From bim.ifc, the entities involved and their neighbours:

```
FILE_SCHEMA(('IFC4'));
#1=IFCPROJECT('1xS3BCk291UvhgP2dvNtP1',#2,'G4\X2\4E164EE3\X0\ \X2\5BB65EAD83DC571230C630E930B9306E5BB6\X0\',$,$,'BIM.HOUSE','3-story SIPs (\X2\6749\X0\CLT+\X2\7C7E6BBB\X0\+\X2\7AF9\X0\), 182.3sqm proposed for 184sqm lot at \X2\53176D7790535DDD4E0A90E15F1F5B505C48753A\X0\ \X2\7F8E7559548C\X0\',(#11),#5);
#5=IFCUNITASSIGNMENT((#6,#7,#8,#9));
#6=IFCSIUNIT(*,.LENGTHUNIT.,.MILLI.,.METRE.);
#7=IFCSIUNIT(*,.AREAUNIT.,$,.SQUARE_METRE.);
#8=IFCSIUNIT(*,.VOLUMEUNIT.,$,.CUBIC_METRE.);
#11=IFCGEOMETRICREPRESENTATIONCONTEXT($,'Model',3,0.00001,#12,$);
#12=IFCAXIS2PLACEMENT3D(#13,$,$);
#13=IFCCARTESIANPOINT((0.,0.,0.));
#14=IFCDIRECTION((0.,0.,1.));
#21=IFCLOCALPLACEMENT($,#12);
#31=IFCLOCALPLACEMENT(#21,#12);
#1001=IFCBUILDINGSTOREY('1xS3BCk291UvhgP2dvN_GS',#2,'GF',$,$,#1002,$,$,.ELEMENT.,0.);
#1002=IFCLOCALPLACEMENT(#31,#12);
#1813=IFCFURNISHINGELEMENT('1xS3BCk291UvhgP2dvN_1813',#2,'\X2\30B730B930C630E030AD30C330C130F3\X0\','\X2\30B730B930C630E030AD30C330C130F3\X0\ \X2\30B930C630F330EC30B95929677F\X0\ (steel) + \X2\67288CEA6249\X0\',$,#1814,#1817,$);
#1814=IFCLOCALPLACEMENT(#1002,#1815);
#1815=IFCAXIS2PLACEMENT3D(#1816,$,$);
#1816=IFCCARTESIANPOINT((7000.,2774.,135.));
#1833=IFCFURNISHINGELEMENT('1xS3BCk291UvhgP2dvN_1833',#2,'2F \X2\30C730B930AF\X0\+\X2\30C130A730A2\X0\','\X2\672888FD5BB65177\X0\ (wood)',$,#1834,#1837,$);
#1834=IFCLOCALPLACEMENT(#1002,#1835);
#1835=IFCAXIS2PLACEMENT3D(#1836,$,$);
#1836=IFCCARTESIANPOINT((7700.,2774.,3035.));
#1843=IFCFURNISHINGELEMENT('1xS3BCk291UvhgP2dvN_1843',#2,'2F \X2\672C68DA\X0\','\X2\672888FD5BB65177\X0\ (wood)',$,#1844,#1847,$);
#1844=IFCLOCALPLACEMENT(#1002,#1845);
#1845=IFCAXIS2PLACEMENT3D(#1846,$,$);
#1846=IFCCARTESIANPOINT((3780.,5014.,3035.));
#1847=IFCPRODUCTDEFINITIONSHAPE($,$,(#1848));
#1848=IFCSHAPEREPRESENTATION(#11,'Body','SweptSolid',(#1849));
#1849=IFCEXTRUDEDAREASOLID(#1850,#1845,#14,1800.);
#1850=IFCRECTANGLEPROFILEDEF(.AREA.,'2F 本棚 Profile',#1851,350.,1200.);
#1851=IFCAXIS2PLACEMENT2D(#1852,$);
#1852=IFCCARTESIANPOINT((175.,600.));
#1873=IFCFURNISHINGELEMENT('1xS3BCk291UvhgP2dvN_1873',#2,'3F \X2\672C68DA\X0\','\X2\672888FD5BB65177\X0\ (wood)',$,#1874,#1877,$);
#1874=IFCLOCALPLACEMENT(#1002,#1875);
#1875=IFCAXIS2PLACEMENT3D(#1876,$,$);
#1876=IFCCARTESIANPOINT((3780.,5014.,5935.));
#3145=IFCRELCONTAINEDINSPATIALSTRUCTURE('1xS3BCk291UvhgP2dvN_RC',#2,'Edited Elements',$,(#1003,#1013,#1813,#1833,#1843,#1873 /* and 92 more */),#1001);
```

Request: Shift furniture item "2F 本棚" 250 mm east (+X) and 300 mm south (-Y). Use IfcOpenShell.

```python
import ifcopenshell
import ifcopenshell.api.geometry
import ifcopenshell.util.placement

model = ifcopenshell.open("bim.ifc")

item = model.by_guid("1xS3BCk291UvhgP2dvN_1843")
matrix = ifcopenshell.util.placement.get_local_placement(item.ObjectPlacement)
matrix[0, 3] += 250.0
matrix[1, 3] -= 300.0
ifcopenshell.api.geometry.edit_object_placement(model, product=item, matrix=matrix, is_si=False)

print(ifcopenshell.util.placement.get_local_placement(item.ObjectPlacement).round(3) + 0.0)

model.write("bim_v2.ifc")
```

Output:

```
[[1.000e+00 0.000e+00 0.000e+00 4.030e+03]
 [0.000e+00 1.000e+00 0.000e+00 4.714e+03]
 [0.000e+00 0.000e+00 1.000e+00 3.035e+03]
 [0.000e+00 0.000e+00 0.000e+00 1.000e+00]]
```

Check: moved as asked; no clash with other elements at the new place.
